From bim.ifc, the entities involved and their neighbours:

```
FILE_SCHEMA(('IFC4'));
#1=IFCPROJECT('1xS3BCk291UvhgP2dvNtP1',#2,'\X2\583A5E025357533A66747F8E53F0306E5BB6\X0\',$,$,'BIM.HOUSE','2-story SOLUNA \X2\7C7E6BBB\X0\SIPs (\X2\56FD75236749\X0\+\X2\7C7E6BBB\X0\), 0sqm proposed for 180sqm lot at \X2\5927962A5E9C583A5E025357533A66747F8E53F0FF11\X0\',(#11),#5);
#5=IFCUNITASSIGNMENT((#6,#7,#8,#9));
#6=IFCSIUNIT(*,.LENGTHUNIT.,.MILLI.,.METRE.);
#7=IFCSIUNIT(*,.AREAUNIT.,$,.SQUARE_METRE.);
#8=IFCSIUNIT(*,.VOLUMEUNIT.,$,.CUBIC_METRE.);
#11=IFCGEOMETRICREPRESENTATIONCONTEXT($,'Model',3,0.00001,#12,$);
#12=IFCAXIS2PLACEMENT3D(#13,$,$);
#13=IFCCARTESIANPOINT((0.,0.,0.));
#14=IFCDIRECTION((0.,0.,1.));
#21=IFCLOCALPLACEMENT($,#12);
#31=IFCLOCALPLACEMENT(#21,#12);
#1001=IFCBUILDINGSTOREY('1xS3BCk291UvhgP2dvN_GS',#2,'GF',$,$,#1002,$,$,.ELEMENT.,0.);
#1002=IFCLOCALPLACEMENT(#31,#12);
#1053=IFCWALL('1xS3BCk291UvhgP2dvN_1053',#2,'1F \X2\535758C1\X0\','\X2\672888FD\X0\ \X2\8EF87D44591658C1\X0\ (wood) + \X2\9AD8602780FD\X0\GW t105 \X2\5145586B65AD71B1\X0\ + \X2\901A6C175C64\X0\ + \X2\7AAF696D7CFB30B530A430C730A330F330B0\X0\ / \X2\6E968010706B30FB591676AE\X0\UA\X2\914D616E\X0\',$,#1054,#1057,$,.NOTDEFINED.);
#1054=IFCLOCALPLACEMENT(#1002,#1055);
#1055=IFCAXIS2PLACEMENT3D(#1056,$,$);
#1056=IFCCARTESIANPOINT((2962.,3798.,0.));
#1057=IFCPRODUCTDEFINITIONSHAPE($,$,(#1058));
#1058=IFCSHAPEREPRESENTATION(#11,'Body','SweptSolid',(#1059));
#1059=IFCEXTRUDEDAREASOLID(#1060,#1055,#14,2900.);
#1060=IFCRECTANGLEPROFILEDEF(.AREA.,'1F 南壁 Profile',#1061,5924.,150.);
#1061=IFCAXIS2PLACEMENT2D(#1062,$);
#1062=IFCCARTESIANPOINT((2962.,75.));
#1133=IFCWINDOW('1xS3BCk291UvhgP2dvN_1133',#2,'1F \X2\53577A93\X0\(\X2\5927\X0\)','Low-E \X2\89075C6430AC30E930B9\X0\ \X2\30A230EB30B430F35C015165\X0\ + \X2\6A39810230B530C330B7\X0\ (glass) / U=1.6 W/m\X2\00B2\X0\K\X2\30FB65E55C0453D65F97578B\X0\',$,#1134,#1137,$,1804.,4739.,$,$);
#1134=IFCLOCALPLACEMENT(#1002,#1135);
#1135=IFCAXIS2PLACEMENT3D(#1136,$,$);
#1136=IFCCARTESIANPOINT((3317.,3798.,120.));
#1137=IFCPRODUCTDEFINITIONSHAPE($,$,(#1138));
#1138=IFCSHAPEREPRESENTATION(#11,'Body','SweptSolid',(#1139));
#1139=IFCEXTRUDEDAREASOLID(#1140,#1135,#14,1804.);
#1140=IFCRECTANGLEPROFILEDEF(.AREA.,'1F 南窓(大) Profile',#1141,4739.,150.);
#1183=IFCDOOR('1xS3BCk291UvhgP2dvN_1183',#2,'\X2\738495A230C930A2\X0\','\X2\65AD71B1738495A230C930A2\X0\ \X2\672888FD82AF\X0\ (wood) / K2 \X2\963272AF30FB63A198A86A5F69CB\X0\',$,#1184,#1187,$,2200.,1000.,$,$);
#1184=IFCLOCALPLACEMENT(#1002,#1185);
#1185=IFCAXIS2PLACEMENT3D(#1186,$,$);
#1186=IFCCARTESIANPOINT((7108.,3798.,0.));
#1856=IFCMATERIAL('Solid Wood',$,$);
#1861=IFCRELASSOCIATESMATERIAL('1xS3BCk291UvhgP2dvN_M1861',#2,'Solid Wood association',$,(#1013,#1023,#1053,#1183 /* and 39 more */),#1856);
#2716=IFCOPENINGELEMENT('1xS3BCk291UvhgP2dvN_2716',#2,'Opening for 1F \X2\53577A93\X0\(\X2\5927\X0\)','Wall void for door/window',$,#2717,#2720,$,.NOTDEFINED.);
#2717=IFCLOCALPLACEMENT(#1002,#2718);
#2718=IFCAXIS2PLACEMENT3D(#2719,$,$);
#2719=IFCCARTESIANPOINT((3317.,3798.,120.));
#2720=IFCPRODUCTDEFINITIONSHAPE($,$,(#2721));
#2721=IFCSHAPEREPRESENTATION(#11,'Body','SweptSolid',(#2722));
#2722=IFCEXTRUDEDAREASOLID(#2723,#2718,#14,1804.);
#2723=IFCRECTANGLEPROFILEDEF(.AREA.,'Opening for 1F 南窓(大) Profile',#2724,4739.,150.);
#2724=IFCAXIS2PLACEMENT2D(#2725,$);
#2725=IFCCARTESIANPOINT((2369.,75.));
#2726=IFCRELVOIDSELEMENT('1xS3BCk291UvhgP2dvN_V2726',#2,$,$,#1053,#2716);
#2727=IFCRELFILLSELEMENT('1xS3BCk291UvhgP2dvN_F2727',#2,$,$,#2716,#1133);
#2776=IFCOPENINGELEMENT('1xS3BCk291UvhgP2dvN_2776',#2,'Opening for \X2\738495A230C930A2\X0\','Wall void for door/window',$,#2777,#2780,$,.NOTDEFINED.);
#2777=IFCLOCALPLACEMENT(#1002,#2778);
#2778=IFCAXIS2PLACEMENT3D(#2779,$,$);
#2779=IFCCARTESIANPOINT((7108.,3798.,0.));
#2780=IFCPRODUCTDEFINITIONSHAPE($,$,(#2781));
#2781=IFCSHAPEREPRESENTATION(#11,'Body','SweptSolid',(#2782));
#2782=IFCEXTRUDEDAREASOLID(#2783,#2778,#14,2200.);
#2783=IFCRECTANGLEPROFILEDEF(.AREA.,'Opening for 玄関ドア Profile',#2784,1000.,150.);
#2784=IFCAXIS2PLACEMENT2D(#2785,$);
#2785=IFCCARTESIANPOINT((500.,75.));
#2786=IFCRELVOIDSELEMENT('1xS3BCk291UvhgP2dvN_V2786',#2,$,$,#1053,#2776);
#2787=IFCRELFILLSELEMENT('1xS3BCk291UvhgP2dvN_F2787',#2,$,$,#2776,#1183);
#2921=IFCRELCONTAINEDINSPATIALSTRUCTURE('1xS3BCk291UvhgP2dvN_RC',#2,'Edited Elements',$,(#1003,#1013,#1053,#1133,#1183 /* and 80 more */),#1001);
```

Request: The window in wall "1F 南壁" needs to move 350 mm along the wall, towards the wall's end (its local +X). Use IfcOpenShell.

```python
import ifcopenshell
import ifcopenshell.api.geometry
import ifcopenshell.util.placement
import ifcopenshell.util.unit

model = ifcopenshell.open("bim.ifc")
unit_scale = ifcopenshell.util.unit.calculate_unit_scale(model)

window = model.by_guid("1xS3BCk291UvhgP2dvN_1133")
opening = window.FillsVoids[0].RelatingOpeningElement
wall = opening.VoidsElements[0].RelatingBuildingElement

wall_matrix = ifcopenshell.util.placement.get_local_placement(wall.ObjectPlacement)
shift = wall_matrix[:3, 0] * 0.35 / unit_scale
before = ifcopenshell.util.placement.get_local_placement(window.ObjectPlacement)[:3, 3].copy()

# The window is not placed relative to its opening, so move both.
for product in (opening, window):
    matrix = ifcopenshell.util.placement.get_local_placement(product.ObjectPlacement)
    matrix[:3, 3] += shift
    ifcopenshell.api.geometry.edit_object_placement(model, product=product, matrix=matrix, is_si=False)

after = ifcopenshell.util.placement.get_local_placement(window.ObjectPlacement)[:3, 3]
print("window moved by", (after - before).round(3) + 0.0)

model.write("bim-out.ifc")
```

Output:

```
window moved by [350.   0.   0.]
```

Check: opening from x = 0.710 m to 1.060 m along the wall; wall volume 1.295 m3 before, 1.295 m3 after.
